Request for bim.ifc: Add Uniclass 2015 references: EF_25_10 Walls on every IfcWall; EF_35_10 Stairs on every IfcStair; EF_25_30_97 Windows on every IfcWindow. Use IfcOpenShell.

First a look at what the model holds.

```python
import ifcopenshell

model = ifcopenshell.open("bim.ifc")
print(model.schema)
print("classifications:", [c.Name for c in model.by_type("IfcClassification")])
for ifc_class in ("IfcDoor", "IfcRoof", "IfcStair", "IfcWall", "IfcWindow"):
    print(ifc_class, len(model.by_type(ifc_class)))
```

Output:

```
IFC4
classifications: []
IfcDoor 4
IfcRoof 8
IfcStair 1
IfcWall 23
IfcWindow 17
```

```python
import ifcopenshell
import ifcopenshell.api.classification

model = ifcopenshell.open("bim.ifc")

system = ifcopenshell.api.classification.add_classification(model, classification="Uniclass 2015")

codes = {
    "IfcWall": ("EF_25_10", "Walls"),
    "IfcStair": ("EF_35_10", "Stairs"),
    "IfcWindow": ("EF_25_30_97", "Windows"),
}
for ifc_class, (code, name) in codes.items():
    products = model.by_type(ifc_class)
    ifcopenshell.api.classification.add_reference(
        model, products=products, classification=system, identification=code, name=name
    )
    print(code, len(products))

model.write("bim_v2.ifc")
```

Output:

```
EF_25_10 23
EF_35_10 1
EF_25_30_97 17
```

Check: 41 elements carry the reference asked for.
